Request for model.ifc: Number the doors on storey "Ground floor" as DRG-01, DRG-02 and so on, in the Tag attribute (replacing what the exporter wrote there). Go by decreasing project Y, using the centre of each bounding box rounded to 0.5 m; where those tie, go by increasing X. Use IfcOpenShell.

First a look at what the model holds.

```python
import ifcopenshell
import ifcopenshell.util.element
import ifcopenshell.util.placement

model = ifcopenshell.open("model.ifc")
print(model.schema)
storey = next(s for s in model.by_type("IfcBuildingStorey") if s.Name == "Ground floor")
doors = [e for e in ifcopenshell.util.element.get_decomposition(storey) if e.is_a("IfcDoor")]
for e in sorted(doors, key=lambda e: e.id()):
    origin = ifcopenshell.util.placement.get_local_placement(e.ObjectPlacement)[:3, 3]
    print(e.id(), e.Tag, e.Name, origin.round(2) + 0.0, sep=" | ")
```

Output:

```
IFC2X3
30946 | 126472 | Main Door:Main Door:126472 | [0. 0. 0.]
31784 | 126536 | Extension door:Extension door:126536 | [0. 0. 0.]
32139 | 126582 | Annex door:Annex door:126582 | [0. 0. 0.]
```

```python
import ifcopenshell
import ifcopenshell.geom
import ifcopenshell.util.element
import ifcopenshell.util.shape

model = ifcopenshell.open("model.ifc")
settings = ifcopenshell.geom.settings()
settings.set("use-world-coords", True)


def centre(element):
    shape = ifcopenshell.geom.create_shape(settings, element)
    return ifcopenshell.util.shape.get_bbox_centroid(shape.geometry)


storey = next(s for s in model.by_type("IfcBuildingStorey") if s.Name == "Ground floor")
doors = [e for e in ifcopenshell.util.element.get_decomposition(storey) if e.is_a("IfcDoor")]

# Insertion points can sit at a corner or the storey origin, so sort by the geometry (in metres).
centres = {e: centre(e) for e in doors}
doors.sort(key=lambda e: (-round(centres[e][1] / 0.5), centres[e][0]))

for i, e in enumerate(doors, start=1):
    number = f"DRG-{i:02d}"
    e.Tag = number
    print(e.id(), number)

model.write("model_updated.ifc")
```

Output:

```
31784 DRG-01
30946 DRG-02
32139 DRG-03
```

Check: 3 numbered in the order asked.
